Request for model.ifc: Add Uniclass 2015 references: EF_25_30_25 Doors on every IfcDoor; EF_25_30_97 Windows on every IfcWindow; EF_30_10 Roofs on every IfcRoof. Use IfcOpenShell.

First a look at what the model holds.

```python
import ifcopenshell

model = ifcopenshell.open("model.ifc")
print(model.schema)
print("classifications:", [c.Name for c in model.by_type("IfcClassification")])
for ifc_class in ("IfcDoor", "IfcRoof", "IfcStair", "IfcWall", "IfcWindow"):
    print(ifc_class, len(model.by_type(ifc_class)))
```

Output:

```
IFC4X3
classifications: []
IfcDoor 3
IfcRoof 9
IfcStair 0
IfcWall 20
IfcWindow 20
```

```python
import ifcopenshell
import ifcopenshell.api.classification

model = ifcopenshell.open("model.ifc")

system = ifcopenshell.api.classification.add_classification(model, classification="Uniclass 2015")

codes = {
    "IfcDoor": ("EF_25_30_25", "Doors"),
    "IfcWindow": ("EF_25_30_97", "Windows"),
    "IfcRoof": ("EF_30_10", "Roofs"),
}
for ifc_class, (code, name) in codes.items():
    products = model.by_type(ifc_class)
    ifcopenshell.api.classification.add_reference(
        model, products=products, classification=system, identification=code, name=name
    )
    print(code, len(products))

model.write("model_rev.ifc")
```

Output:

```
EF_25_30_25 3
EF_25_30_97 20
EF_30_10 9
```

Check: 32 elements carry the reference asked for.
